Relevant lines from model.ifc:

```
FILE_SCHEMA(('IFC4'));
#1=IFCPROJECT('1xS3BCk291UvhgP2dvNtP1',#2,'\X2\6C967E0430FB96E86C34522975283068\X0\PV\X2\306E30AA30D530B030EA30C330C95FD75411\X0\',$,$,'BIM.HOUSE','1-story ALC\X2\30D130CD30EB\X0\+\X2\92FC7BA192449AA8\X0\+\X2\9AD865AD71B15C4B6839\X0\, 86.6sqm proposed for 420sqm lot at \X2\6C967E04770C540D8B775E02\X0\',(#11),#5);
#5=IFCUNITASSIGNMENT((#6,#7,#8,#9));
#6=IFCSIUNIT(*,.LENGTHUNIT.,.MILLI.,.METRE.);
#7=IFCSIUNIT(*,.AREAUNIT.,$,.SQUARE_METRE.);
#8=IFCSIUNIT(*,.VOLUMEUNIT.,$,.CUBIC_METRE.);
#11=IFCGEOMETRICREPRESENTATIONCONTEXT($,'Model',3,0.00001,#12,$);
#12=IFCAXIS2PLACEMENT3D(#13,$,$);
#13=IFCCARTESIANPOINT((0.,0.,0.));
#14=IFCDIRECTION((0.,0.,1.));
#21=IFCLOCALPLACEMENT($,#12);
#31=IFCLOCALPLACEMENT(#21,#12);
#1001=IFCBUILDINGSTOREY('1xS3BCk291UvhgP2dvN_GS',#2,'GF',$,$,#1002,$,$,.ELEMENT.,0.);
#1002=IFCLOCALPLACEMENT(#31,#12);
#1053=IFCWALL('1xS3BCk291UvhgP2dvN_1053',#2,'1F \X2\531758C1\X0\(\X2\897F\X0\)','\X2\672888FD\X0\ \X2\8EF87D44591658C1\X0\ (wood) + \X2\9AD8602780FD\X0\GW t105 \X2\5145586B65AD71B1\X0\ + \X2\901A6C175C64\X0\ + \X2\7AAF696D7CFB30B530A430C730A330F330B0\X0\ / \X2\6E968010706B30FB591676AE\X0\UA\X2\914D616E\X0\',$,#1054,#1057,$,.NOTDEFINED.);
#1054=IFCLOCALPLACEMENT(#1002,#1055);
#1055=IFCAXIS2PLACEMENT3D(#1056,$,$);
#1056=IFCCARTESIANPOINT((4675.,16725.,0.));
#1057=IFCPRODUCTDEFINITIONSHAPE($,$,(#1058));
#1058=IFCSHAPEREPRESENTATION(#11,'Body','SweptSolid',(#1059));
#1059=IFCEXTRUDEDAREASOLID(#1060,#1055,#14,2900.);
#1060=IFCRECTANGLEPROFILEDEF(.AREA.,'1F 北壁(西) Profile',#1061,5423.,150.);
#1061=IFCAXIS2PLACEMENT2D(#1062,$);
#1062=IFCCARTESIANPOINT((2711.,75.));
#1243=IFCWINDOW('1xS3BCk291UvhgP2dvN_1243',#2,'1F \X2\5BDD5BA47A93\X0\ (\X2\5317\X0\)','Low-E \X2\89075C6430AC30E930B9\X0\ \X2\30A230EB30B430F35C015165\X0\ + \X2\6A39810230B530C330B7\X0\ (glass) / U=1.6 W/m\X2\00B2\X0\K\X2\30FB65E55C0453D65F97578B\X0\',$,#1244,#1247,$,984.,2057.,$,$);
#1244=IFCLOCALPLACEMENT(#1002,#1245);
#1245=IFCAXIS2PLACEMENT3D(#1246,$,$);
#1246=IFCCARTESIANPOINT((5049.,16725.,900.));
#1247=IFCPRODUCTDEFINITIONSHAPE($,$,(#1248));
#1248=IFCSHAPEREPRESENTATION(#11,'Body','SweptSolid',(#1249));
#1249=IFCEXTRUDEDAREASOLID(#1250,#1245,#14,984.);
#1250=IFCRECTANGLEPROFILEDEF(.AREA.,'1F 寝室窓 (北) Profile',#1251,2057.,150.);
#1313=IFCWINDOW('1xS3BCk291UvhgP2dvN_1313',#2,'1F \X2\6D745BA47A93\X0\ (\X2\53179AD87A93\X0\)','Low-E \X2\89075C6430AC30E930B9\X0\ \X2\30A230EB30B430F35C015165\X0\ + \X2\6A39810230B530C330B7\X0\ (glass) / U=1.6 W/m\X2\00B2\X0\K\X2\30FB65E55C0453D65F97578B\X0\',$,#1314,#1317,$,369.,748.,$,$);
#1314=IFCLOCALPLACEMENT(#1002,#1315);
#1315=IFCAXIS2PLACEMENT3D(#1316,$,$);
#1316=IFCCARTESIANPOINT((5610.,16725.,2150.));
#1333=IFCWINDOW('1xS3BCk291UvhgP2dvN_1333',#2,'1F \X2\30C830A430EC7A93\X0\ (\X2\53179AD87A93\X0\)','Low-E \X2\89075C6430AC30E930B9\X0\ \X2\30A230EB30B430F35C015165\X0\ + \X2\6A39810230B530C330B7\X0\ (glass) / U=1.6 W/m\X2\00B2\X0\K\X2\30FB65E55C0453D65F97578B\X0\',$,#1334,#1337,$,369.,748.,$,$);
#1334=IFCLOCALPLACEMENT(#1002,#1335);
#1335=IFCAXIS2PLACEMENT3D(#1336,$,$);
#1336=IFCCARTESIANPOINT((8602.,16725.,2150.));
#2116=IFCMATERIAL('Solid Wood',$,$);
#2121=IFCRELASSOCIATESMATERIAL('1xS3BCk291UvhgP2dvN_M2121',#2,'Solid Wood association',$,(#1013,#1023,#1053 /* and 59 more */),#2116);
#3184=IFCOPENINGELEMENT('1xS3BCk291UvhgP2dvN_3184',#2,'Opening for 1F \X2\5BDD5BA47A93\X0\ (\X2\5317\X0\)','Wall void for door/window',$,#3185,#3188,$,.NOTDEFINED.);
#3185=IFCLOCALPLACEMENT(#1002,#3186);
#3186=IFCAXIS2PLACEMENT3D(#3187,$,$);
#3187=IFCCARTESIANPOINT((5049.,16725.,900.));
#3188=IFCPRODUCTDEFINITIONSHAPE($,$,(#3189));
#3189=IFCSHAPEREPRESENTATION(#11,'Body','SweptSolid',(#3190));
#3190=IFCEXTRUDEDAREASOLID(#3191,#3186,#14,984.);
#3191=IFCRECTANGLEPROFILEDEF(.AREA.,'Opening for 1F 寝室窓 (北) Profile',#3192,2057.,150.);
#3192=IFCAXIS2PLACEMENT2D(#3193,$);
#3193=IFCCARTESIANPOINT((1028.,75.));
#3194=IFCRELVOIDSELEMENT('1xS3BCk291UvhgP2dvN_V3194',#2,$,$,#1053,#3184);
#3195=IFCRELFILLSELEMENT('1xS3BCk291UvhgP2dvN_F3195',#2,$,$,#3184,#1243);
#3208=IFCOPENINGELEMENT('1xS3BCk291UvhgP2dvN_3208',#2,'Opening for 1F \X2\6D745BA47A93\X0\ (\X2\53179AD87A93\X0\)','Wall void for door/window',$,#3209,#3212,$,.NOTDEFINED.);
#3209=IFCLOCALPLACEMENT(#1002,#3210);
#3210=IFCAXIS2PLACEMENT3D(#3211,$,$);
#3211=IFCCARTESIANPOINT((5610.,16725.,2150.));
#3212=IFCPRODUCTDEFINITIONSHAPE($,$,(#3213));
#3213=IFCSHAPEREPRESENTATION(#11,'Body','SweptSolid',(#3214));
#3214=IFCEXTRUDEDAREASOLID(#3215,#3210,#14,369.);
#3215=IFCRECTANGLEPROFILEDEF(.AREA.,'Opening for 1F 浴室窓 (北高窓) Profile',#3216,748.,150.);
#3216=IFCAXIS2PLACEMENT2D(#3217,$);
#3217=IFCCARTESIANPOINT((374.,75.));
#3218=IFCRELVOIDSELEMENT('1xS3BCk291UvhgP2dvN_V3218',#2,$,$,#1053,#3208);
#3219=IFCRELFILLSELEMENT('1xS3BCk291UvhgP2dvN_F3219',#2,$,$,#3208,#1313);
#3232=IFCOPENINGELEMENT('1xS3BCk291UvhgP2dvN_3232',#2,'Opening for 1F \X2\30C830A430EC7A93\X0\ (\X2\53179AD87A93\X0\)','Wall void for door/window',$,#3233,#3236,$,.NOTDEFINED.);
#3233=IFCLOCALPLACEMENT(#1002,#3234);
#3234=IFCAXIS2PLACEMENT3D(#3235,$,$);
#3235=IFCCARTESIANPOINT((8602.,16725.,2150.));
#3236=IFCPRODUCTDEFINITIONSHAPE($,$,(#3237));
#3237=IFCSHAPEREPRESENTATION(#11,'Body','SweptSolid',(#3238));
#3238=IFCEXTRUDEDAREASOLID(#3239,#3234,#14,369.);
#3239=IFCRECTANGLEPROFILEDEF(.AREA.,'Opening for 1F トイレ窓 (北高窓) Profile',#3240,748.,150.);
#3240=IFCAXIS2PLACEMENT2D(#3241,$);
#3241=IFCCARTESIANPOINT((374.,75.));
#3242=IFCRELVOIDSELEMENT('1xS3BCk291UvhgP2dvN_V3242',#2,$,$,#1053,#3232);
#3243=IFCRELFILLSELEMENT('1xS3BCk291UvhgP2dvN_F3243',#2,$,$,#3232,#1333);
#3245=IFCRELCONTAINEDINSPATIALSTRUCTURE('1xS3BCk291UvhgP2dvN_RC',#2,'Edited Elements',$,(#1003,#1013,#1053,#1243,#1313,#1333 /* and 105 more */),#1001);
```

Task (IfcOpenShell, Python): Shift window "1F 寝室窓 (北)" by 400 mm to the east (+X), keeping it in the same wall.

```python
import ifcopenshell
import ifcopenshell.api.geometry
import ifcopenshell.util.placement
import ifcopenshell.util.unit

model = ifcopenshell.open("model.ifc")
unit_scale = ifcopenshell.util.unit.calculate_unit_scale(model)

window = model.by_guid("1xS3BCk291UvhgP2dvN_1243")
opening = window.FillsVoids[0].RelatingOpeningElement
wall = opening.VoidsElements[0].RelatingBuildingElement

wall_matrix = ifcopenshell.util.placement.get_local_placement(wall.ObjectPlacement)
shift = wall_matrix[:3, 0] * 0.4 / unit_scale
before = ifcopenshell.util.placement.get_local_placement(window.ObjectPlacement)[:3, 3].copy()

# The window is not placed relative to its opening, so move both.
for product in (opening, window):
    matrix = ifcopenshell.util.placement.get_local_placement(product.ObjectPlacement)
    matrix[:3, 3] += shift
    ifcopenshell.api.geometry.edit_object_placement(model, product=product, matrix=matrix, is_si=False)

after = ifcopenshell.util.placement.get_local_placement(window.ObjectPlacement)[:3, 3]
print("window moved by", (after - before).round(3) + 0.0)

model.write("model-out.ifc")
```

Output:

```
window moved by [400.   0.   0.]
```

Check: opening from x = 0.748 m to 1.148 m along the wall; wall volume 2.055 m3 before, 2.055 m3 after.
